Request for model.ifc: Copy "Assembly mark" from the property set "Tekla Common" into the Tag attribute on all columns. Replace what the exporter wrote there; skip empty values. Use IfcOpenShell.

First a look at what the model holds.

```python
import ifcopenshell
import ifcopenshell.util.element

model = ifcopenshell.open("model.ifc")
print(model.schema)
columns = model.by_type("IfcColumn")
print(len(columns), "columns")
for e in columns[:8]:
    source = ifcopenshell.util.element.get_pset(e, "Tekla Common", "Assembly mark")
    target = e.Tag
    print(e.id(), repr(source), repr(target), sep=" | ")
```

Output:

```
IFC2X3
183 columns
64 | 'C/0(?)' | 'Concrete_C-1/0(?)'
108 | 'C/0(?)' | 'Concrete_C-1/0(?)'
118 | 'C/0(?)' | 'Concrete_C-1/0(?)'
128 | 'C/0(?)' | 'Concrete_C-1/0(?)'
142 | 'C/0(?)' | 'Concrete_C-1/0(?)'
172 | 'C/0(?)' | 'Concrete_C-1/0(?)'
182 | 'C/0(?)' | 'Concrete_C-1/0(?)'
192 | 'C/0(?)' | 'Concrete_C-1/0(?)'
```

```python
import ifcopenshell
import ifcopenshell.util.element

model = ifcopenshell.open("model.ifc")

count = 0
for e in model.by_type("IfcColumn"):
    value = ifcopenshell.util.element.get_pset(e, "Tekla Common", "Assembly mark")
    current = e.Tag
    if not value or not value.strip() or current == value:
        continue
    e.Tag = value
    count += 1

print(count, "columns updated")

model.write("model_v2.ifc")
```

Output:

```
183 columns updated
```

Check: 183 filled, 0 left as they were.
